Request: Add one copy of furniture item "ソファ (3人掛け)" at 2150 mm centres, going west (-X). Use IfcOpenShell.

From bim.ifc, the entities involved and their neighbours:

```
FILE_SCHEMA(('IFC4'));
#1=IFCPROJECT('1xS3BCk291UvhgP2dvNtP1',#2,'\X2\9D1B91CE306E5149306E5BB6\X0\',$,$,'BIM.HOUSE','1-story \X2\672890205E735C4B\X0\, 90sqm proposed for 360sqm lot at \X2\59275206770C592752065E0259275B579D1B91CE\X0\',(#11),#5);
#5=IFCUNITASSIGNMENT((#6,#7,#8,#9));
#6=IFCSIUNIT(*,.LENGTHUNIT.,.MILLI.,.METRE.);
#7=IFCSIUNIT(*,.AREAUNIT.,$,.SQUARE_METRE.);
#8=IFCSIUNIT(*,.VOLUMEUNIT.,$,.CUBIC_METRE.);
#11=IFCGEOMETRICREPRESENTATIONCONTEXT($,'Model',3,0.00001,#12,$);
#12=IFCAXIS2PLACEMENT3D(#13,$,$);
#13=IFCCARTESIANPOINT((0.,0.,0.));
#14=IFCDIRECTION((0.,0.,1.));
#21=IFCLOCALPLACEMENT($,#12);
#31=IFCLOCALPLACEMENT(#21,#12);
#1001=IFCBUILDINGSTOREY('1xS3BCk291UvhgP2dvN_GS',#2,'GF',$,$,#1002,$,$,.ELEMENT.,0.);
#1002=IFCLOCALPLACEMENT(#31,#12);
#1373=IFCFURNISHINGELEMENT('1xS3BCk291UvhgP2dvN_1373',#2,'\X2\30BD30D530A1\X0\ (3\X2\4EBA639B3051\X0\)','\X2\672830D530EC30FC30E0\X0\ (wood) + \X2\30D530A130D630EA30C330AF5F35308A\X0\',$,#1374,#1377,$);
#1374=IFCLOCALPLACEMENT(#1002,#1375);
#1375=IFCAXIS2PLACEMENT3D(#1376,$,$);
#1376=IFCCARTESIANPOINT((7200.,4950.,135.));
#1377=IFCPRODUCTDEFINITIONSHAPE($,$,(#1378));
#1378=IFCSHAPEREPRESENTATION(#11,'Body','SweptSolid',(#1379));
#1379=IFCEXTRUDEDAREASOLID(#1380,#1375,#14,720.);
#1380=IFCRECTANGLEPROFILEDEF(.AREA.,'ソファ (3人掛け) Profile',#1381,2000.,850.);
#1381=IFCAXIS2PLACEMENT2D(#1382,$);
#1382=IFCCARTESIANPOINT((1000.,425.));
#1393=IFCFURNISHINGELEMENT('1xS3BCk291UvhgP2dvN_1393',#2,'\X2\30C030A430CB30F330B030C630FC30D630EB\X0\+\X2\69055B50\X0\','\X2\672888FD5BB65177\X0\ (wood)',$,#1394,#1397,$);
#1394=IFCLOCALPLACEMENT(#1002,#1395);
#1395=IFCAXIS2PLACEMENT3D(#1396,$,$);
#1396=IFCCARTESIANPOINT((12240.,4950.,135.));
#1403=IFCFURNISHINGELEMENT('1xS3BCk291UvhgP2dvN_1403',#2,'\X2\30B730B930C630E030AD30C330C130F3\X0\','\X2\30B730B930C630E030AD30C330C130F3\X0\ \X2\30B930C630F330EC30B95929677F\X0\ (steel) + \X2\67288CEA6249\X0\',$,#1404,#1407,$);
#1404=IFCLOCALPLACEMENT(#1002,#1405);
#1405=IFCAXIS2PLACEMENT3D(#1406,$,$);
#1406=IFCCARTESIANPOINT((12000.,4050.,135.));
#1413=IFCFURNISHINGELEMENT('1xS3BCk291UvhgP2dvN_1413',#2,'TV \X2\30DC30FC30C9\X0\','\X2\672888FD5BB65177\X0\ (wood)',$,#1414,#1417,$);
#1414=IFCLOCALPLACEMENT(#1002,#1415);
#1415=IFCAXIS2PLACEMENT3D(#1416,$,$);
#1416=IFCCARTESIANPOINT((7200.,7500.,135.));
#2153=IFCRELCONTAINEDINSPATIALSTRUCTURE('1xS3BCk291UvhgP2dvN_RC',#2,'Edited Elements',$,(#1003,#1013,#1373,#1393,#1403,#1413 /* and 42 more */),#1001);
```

```python
import numpy as np
import ifcopenshell
import ifcopenshell.api.geometry
import ifcopenshell.api.root
import ifcopenshell.util.element
import ifcopenshell.util.placement
import ifcopenshell.util.unit

model = ifcopenshell.open("bim.ifc")
unit_scale = ifcopenshell.util.unit.calculate_unit_scale(model)


def reuse_history(source, copy):
    """copy_class also copies each property set's owner history, people and application; keep the originals."""
    for rel in copy.IsDefinedBy:
        if rel.is_a("IfcRelDefinesByProperties") and (history := rel.RelatingPropertyDefinition.OwnerHistory):
            rel.RelatingPropertyDefinition.OwnerHistory = source.OwnerHistory
            ifcopenshell.util.element.remove_deep2(model, history)


source = model.by_id(1373)
base = ifcopenshell.util.placement.get_local_placement(source.ObjectPlacement)
step = np.array([-1.0, 0.0, 0.0]) * 2.15 / unit_scale

for i in range(1, 2):
    copy = ifcopenshell.api.root.copy_class(model, product=source)
    copy.Representation = ifcopenshell.util.element.copy_deep(
        model, source.Representation, exclude=["IfcGeometricRepresentationContext", "IfcRepresentationMap"]
    )
    reuse_history(source, copy)
    matrix = base.copy()
    matrix[:3, 3] += i * step
    print("added at", matrix[:3, 3].round(3) + 0.0)
    ifcopenshell.api.geometry.edit_object_placement(model, product=copy, matrix=matrix, is_si=False)

model.write("bim-out.ifc")
```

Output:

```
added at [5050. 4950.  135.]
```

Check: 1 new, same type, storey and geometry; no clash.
